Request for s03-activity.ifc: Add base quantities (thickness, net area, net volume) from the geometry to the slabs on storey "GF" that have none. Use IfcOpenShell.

First a look at what the model holds.

```python
import ifcopenshell
import ifcopenshell.util.element
import ifcopenshell.util.unit

model = ifcopenshell.open("s03-activity.ifc")
print(model.schema)
for unit_type in ("LENGTHUNIT", "AREAUNIT", "VOLUMEUNIT"):
    print(unit_type, ifcopenshell.util.unit.calculate_unit_scale(model, unit_type))
storey = next(s for s in model.by_type("IfcBuildingStorey") if s.Name == "GF")
slabs = [e for e in ifcopenshell.util.element.get_decomposition(storey) if e.is_a("IfcSlab")]
for e in sorted(slabs, key=lambda e: e.id()):
    print(e.id(), e.is_a(), e.Name, list(ifcopenshell.util.element.get_psets(e, qtos_only=True)), sep=" | ")
```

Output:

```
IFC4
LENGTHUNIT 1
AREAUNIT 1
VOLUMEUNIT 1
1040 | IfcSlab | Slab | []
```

```python
import ifcopenshell
import ifcopenshell.api.pset
import ifcopenshell.geom
import ifcopenshell.util.element
import ifcopenshell.util.shape
import ifcopenshell.util.unit

model = ifcopenshell.open("s03-activity.ifc")
unit_scale = ifcopenshell.util.unit.calculate_unit_scale(model)
area_scale = ifcopenshell.util.unit.calculate_unit_scale(model, "AREAUNIT")
volume_scale = ifcopenshell.util.unit.calculate_unit_scale(model, "VOLUMEUNIT")
settings = ifcopenshell.geom.settings()

storey = next(s for s in model.by_type("IfcBuildingStorey") if s.Name == "GF")
slabs = [e for e in ifcopenshell.util.element.get_decomposition(storey) if e.is_a("IfcSlab")]

for e in sorted(slabs, key=lambda e: e.id()):
    if ifcopenshell.util.element.get_psets(e, qtos_only=True, should_inherit=False):
        continue
    # Geometry comes back in metres, in the element's own axes.
    shape = ifcopenshell.geom.create_shape(settings, e)
    values = {
        "Width": ifcopenshell.util.shape.get_z(shape.geometry) / unit_scale,
        "NetArea": ifcopenshell.util.shape.get_footprint_area(shape.geometry) / area_scale,
        "NetVolume": ifcopenshell.util.shape.get_volume(shape.geometry) / volume_scale,
    }
    qto = ifcopenshell.api.pset.add_qto(model, product=e, name="Qto_SlabBaseQuantities")
    ifcopenshell.api.pset.edit_qto(model, qto=qto, properties=values)
    print(e.id(), {k: round(v, 3) for k, v in values.items()})

model.write("s03-activity-out.ifc")
```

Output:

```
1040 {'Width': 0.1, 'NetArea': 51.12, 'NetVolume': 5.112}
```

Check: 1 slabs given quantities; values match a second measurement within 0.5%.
